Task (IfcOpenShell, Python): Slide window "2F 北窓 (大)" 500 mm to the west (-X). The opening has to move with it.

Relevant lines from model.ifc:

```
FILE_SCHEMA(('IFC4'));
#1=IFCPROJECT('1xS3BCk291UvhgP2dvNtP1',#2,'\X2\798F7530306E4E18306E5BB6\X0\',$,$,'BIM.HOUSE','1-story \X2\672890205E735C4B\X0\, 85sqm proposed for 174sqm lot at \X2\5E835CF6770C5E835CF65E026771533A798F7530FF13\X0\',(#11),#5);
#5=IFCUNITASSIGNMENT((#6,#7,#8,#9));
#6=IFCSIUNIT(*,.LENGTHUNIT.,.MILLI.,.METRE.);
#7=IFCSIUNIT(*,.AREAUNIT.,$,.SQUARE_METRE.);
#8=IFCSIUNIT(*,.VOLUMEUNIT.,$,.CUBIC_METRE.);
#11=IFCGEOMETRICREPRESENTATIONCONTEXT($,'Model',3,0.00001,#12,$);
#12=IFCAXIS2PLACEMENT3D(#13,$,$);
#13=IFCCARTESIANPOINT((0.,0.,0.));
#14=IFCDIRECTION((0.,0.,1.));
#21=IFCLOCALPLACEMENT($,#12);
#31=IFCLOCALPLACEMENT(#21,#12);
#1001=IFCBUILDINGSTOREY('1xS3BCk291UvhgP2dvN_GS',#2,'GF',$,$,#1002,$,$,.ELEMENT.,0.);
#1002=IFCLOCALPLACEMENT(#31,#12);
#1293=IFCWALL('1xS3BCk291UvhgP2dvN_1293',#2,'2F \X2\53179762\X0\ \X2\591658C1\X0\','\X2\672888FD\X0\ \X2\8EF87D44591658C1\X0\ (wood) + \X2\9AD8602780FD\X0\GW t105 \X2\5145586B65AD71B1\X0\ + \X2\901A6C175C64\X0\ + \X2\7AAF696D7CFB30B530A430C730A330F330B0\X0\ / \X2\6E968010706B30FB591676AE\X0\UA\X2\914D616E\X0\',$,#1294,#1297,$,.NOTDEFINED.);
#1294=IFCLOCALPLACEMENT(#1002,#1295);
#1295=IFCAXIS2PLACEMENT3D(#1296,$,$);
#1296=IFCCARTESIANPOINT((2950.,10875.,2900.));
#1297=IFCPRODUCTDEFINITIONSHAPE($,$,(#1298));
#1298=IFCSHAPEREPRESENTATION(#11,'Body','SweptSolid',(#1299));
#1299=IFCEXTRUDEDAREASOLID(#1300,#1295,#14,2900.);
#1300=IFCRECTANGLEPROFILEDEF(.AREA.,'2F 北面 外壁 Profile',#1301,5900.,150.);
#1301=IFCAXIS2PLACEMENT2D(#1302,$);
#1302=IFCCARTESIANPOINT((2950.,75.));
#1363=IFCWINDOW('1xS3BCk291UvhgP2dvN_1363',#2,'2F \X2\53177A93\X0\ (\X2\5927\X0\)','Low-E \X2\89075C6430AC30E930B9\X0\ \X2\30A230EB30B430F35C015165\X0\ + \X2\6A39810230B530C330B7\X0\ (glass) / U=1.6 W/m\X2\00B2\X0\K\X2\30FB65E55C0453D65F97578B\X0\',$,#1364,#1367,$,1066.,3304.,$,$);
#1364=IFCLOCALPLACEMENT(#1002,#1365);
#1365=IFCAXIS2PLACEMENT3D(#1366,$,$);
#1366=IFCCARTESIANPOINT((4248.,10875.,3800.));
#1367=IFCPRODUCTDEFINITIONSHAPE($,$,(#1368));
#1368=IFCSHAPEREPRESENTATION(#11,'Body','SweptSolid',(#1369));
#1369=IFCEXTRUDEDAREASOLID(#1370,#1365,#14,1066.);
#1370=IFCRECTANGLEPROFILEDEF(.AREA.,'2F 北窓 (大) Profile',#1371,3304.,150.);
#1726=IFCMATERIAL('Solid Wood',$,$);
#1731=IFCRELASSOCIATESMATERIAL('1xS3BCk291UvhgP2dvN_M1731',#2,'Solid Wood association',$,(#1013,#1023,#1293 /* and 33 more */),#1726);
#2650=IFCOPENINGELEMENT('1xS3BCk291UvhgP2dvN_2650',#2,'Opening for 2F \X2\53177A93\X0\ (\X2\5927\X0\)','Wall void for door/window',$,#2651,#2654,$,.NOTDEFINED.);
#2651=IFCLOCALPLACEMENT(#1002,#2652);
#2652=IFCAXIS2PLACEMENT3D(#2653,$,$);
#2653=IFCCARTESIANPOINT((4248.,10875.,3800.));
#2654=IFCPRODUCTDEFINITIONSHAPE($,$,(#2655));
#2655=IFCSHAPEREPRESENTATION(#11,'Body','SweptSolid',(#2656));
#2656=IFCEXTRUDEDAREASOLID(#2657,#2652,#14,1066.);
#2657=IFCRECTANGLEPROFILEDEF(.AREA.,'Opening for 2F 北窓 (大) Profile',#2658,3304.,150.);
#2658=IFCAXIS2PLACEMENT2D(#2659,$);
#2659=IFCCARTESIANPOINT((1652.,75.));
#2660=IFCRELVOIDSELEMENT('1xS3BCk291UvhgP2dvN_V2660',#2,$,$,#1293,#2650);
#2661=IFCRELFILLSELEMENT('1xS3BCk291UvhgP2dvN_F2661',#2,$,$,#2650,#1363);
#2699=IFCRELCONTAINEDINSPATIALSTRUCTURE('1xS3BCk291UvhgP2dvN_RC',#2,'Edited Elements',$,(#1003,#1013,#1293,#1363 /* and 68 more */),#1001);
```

```python
import ifcopenshell
import ifcopenshell.api.geometry
import ifcopenshell.util.placement
import ifcopenshell.util.unit

model = ifcopenshell.open("model.ifc")
unit_scale = ifcopenshell.util.unit.calculate_unit_scale(model)

window = model.by_guid("1xS3BCk291UvhgP2dvN_1363")
opening = window.FillsVoids[0].RelatingOpeningElement
wall = opening.VoidsElements[0].RelatingBuildingElement

wall_matrix = ifcopenshell.util.placement.get_local_placement(wall.ObjectPlacement)
shift = wall_matrix[:3, 0] * -0.5 / unit_scale
before = ifcopenshell.util.placement.get_local_placement(window.ObjectPlacement)[:3, 3].copy()

# The window is not placed relative to its opening, so move both.
for product in (opening, window):
    matrix = ifcopenshell.util.placement.get_local_placement(product.ObjectPlacement)
    matrix[:3, 3] += shift
    ifcopenshell.api.geometry.edit_object_placement(model, product=product, matrix=matrix, is_si=False)

after = ifcopenshell.util.placement.get_local_placement(window.ObjectPlacement)[:3, 3]
print("window moved by", (after - before).round(3) + 0.0)

model.write("model_rev.ifc")
```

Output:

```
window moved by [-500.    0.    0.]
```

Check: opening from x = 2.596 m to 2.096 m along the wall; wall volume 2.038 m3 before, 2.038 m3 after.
